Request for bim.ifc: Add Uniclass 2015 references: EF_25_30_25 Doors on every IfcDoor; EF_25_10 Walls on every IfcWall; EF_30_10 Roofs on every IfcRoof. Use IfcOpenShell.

First a look at what the model holds.

```python
import ifcopenshell

model = ifcopenshell.open("bim.ifc")
print(model.schema)
print("classifications:", [c.Name for c in model.by_type("IfcClassification")])
for ifc_class in ("IfcDoor", "IfcRoof", "IfcStair", "IfcWall", "IfcWindow"):
    print(ifc_class, len(model.by_type(ifc_class)))
```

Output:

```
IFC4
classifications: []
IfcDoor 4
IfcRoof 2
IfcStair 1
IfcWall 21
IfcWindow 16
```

```python
import ifcopenshell
import ifcopenshell.api.classification

model = ifcopenshell.open("bim.ifc")

system = ifcopenshell.api.classification.add_classification(model, classification="Uniclass 2015")

codes = {
    "IfcDoor": ("EF_25_30_25", "Doors"),
    "IfcWall": ("EF_25_10", "Walls"),
    "IfcRoof": ("EF_30_10", "Roofs"),
}
for ifc_class, (code, name) in codes.items():
    products = model.by_type(ifc_class)
    ifcopenshell.api.classification.add_reference(
        model, products=products, classification=system, identification=code, name=name
    )
    print(code, len(products))

model.write("bim-out.ifc")
```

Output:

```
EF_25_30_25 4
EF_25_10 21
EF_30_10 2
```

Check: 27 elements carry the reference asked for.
